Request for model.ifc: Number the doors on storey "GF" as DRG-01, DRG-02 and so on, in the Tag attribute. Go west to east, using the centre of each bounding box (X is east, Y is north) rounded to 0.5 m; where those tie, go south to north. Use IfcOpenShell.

First a look at what the model holds.

```python
import ifcopenshell
import ifcopenshell.util.element
import ifcopenshell.util.placement

model = ifcopenshell.open("model.ifc")
print(model.schema)
storey = next(s for s in model.by_type("IfcBuildingStorey") if s.Name == "GF")
doors = [e for e in ifcopenshell.util.element.get_decomposition(storey) if e.is_a("IfcDoor")]
for e in sorted(doors, key=lambda e: e.id()):
    origin = ifcopenshell.util.placement.get_local_placement(e.ObjectPlacement)[:3, 3]
    print(e.id(), e.Tag, e.Name, origin.round(2) + 0.0, sep=" | ")
```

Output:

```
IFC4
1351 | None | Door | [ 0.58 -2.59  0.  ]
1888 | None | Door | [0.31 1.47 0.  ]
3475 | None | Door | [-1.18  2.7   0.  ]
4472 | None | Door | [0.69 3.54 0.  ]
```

```python
import ifcopenshell
import ifcopenshell.geom
import ifcopenshell.util.element
import ifcopenshell.util.shape

model = ifcopenshell.open("model.ifc")
settings = ifcopenshell.geom.settings()
settings.set("use-world-coords", True)


def centre(element):
    shape = ifcopenshell.geom.create_shape(settings, element)
    return ifcopenshell.util.shape.get_bbox_centroid(shape.geometry)


storey = next(s for s in model.by_type("IfcBuildingStorey") if s.Name == "GF")
doors = [e for e in ifcopenshell.util.element.get_decomposition(storey) if e.is_a("IfcDoor")]

# Insertion points can sit at a corner or the storey origin, so sort by the geometry (in metres).
centres = {e: centre(e) for e in doors}
doors.sort(key=lambda e: (round(centres[e][0] / 0.5), centres[e][1]))

for i, e in enumerate(doors, start=1):
    number = f"DRG-{i:02d}"
    e.Tag = number
    print(e.id(), number)

model.write("model_rev.ifc")
```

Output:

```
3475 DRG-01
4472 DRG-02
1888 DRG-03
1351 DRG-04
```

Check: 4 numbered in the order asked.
